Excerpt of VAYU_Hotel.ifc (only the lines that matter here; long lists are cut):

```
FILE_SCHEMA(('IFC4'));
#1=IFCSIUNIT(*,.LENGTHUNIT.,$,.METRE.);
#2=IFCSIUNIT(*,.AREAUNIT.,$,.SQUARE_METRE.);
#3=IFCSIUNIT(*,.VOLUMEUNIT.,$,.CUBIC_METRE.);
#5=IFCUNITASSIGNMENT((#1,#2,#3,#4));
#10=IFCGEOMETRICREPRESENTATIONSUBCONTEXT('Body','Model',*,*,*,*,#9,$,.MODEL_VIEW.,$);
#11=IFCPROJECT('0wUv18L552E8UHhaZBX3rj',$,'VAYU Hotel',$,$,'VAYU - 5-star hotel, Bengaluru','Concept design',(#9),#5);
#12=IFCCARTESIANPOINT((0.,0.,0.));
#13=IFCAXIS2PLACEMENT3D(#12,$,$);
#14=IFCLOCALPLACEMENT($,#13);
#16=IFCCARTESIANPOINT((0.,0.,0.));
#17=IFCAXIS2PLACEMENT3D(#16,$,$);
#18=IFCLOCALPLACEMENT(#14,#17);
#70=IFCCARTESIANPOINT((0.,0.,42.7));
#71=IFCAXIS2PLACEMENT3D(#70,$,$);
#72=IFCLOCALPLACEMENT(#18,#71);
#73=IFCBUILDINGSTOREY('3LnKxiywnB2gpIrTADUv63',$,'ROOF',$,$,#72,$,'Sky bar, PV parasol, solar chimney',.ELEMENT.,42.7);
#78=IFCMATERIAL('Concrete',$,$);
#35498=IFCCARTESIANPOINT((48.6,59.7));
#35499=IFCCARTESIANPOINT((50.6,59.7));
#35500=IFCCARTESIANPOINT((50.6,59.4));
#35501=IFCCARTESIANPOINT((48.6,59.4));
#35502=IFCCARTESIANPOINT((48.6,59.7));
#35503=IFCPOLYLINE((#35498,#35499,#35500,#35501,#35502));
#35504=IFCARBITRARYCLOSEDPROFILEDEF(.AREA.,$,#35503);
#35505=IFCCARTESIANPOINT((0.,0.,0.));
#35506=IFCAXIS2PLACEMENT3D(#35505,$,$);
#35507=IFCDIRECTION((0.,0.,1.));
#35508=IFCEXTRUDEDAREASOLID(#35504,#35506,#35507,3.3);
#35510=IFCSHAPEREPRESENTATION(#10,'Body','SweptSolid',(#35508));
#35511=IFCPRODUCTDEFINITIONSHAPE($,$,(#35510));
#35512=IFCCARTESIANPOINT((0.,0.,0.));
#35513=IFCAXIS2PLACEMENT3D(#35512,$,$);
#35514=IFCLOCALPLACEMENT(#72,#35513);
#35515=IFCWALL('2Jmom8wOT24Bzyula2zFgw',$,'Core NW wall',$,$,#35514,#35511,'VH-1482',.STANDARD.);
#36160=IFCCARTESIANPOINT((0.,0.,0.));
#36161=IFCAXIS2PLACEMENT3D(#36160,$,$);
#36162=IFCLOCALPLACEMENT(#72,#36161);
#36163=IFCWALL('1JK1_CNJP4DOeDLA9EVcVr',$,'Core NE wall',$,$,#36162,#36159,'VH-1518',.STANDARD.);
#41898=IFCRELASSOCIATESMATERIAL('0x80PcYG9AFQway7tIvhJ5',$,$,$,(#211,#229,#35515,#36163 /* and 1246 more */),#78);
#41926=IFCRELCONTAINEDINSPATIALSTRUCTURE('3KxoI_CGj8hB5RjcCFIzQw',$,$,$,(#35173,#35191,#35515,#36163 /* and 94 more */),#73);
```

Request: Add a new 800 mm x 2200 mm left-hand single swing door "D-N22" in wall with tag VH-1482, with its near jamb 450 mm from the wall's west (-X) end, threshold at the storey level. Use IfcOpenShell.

```python
import numpy as np
import ifcopenshell
import ifcopenshell.api.feature
import ifcopenshell.api.geometry
import ifcopenshell.api.root
import ifcopenshell.api.spatial
import ifcopenshell.geom
import ifcopenshell.util.element
import ifcopenshell.util.placement
import ifcopenshell.util.representation
import ifcopenshell.util.shape
import ifcopenshell.util.unit

model = ifcopenshell.open("VAYU_Hotel.ifc")
unit_scale = ifcopenshell.util.unit.calculate_unit_scale(model)
settings = ifcopenshell.geom.settings()


def volume(element):
    """Net volume in cubic metres, openings subtracted."""
    shape = ifcopenshell.geom.create_shape(settings, element)
    return ifcopenshell.util.shape.get_volume(shape.geometry)


wall = model.by_guid("2Jmom8wOT24Bzyula2zFgw")
storey = ifcopenshell.util.element.get_container(wall, ifc_class="IfcBuildingStorey")
context = ifcopenshell.util.representation.get_context(model, "Model", "Body", "MODEL_VIEW")
before = volume(wall)

width, height, from_end, sill = 0.8, 2.2, 0.45, 0.0  # metres

# The wall runs along its own X axis, and the end named is its -X end.
wall_shape = ifcopenshell.geom.create_shape(settings, wall)
x, y, z = ifcopenshell.util.shape.get_vertices(wall_shape.geometry).T
start = x.min() + from_end
face, thickness = float(y.min()), float(y.max() - y.min())
wall_matrix = ifcopenshell.util.placement.get_local_placement(wall.ObjectPlacement)
level = ifcopenshell.util.placement.get_local_placement(storey.ObjectPlacement)[2, 3]


def in_wall(x, y):
    """Placement at x, y metres in the wall's axes, at sill height."""
    matrix = wall_matrix.copy()
    matrix[:, 3] = wall_matrix @ np.array([x / unit_scale, y / unit_scale, 0.0, 1.0])
    matrix[2, 3] = level + sill / unit_scale
    return matrix


# Opening: a box that overshoots both wall faces by 50 mm.
opening = ifcopenshell.api.root.create_entity(model, ifc_class="IfcOpeningElement", predefined_type="OPENING")
box = ifcopenshell.api.geometry.add_wall_representation(
    model, context=context, length=width, height=height, thickness=thickness + 0.1
)
ifcopenshell.api.geometry.assign_representation(model, product=opening, representation=box)
ifcopenshell.api.geometry.edit_object_placement(model, product=opening, matrix=in_wall(start, face - 0.05), is_si=False)
ifcopenshell.api.feature.add_feature(model, feature=opening, element=wall)

door = ifcopenshell.api.root.create_entity(model, ifc_class="IfcDoor", name="D-N22", predefined_type="DOOR")
door.OverallWidth, door.OverallHeight = width / unit_scale, height / unit_scale
door.OperationType = "SINGLE_SWING_LEFT"
body = ifcopenshell.api.geometry.add_door_representation(
    model,
    context=context,
    overall_width=door.OverallWidth,
    overall_height=door.OverallHeight,
    operation_type="SINGLE_SWING_LEFT",
    lining_properties={"LiningDepth": thickness / unit_scale, "ThresholdDepth": thickness / unit_scale},
)
ifcopenshell.api.geometry.assign_representation(model, product=door, representation=body)
ifcopenshell.api.spatial.assign_container(model, products=[door], relating_structure=storey)
ifcopenshell.api.feature.add_filling(model, opening=opening, element=door)

# The lining spans the wall, so the door starts at the wall face.
ifcopenshell.api.geometry.edit_object_placement(model, product=door, matrix=in_wall(start, face), is_si=False)

after = volume(wall)

print(f"wall volume {before:.3f} -> {after:.3f} m3")

model.write("VAYU_Hotel_rev.ifc")
```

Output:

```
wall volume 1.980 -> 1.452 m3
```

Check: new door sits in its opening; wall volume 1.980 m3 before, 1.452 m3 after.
